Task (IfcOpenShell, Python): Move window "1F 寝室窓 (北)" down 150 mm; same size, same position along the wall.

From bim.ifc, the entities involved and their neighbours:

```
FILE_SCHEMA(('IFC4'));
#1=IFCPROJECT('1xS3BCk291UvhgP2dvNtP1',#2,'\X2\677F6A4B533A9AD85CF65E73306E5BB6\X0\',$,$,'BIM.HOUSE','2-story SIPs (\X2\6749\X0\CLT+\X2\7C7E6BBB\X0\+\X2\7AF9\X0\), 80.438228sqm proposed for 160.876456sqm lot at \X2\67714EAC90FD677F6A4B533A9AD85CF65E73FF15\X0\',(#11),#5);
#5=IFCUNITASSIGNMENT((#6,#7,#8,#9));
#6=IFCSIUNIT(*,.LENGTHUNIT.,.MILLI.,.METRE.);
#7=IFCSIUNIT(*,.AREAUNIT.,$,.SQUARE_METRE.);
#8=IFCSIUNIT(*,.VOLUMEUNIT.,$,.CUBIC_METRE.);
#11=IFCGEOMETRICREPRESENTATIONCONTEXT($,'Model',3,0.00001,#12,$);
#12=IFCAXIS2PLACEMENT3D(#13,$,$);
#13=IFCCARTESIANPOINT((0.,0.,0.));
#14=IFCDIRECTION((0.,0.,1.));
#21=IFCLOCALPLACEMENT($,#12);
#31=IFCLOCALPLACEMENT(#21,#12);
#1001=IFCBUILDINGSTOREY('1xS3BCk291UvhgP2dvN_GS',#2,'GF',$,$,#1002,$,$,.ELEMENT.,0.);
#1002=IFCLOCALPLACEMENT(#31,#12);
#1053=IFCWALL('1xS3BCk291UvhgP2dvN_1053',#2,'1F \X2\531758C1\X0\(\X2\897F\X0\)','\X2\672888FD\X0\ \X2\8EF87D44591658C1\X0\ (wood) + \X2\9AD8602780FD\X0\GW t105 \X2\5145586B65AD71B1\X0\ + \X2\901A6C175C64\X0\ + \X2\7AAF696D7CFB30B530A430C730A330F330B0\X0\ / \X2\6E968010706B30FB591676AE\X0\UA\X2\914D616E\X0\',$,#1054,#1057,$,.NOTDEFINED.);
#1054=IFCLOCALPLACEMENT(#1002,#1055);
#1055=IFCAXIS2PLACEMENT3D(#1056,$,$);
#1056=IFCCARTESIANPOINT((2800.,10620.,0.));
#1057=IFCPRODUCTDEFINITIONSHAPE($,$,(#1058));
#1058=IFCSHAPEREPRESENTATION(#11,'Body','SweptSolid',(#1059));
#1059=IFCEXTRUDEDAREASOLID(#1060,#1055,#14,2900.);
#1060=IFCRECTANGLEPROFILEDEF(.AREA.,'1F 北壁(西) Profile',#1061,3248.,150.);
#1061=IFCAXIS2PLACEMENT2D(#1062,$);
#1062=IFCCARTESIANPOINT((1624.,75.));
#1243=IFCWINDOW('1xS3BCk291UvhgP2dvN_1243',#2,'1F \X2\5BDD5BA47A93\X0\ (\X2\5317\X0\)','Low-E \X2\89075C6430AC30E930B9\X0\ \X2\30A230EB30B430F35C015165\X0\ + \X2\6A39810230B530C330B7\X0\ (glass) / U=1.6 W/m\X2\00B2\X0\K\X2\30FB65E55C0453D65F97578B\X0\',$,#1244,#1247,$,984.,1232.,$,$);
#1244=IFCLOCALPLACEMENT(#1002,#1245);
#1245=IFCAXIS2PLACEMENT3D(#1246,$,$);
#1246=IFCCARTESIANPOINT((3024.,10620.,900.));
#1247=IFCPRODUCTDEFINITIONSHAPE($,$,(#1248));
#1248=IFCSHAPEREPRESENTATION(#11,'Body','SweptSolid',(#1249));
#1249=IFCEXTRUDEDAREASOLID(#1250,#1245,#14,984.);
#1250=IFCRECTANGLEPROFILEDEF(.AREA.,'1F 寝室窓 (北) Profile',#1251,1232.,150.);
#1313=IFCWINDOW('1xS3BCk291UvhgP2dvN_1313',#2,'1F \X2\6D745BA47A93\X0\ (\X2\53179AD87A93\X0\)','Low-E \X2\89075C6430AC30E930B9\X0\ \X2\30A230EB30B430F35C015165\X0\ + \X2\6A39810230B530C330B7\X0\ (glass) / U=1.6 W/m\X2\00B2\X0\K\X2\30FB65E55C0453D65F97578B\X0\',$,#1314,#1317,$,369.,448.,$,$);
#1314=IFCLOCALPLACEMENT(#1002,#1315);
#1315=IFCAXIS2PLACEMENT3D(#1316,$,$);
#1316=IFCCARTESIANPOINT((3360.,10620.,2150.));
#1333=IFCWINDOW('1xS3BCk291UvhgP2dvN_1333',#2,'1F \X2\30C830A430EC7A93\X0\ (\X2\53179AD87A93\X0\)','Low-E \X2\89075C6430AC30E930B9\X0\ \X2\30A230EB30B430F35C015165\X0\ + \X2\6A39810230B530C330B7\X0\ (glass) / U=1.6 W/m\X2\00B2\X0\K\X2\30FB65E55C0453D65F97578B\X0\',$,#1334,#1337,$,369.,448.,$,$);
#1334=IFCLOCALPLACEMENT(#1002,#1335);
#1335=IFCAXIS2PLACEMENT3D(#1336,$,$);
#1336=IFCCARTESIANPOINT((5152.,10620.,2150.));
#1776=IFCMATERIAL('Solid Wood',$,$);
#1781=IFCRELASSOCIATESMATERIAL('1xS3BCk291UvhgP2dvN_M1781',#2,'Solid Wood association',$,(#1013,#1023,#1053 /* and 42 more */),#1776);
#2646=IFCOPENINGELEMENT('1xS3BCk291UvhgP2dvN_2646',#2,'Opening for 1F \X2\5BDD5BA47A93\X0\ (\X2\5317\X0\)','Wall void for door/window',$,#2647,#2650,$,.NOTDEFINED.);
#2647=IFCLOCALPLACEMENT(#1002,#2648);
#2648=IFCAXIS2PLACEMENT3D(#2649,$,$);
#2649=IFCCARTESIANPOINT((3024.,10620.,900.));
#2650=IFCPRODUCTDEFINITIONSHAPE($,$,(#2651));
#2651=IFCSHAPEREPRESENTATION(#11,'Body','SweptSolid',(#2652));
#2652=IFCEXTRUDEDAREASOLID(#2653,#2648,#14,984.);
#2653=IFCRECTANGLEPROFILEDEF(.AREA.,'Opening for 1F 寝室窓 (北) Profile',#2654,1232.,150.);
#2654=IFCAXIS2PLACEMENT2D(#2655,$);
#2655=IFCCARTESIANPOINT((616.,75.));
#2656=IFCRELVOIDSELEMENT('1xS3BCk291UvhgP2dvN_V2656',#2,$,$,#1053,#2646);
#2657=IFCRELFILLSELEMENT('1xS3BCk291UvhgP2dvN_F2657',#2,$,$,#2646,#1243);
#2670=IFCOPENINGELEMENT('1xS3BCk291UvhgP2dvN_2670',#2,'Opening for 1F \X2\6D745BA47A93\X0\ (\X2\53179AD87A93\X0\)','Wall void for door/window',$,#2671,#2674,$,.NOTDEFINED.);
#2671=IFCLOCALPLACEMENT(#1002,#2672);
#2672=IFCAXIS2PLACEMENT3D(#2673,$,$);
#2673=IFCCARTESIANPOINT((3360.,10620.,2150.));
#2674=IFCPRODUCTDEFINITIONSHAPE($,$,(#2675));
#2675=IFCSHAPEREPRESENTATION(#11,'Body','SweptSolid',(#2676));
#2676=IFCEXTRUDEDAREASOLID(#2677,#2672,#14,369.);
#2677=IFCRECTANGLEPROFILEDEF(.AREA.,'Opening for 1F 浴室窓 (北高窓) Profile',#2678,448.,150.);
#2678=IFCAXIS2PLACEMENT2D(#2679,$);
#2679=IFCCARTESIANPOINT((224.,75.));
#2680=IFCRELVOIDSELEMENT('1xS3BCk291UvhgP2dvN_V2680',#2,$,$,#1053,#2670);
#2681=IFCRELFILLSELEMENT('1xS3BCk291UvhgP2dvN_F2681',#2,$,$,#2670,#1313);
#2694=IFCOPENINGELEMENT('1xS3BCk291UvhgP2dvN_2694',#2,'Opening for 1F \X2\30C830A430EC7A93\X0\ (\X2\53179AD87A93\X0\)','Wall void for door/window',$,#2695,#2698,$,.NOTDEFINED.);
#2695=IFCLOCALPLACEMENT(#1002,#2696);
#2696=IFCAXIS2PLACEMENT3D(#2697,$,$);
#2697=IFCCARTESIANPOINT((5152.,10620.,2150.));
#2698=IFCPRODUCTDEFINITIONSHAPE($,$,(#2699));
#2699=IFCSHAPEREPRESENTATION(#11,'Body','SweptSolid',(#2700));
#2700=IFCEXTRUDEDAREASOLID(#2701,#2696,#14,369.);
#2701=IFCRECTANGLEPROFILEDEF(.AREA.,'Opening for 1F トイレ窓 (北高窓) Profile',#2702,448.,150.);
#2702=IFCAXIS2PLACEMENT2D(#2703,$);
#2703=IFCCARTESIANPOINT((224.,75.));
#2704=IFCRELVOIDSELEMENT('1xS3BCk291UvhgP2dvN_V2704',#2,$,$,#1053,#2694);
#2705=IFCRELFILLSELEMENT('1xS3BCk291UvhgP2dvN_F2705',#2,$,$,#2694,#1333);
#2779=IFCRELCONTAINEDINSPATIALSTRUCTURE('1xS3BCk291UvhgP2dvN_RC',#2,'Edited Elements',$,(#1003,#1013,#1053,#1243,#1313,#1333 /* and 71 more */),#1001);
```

```python
import numpy as np
import ifcopenshell
import ifcopenshell.api.geometry
import ifcopenshell.util.placement
import ifcopenshell.util.unit

model = ifcopenshell.open("bim.ifc")
unit_scale = ifcopenshell.util.unit.calculate_unit_scale(model)

window = model.by_guid("1xS3BCk291UvhgP2dvN_1243")
opening = window.FillsVoids[0].RelatingOpeningElement
dz = -0.15 / unit_scale

shift = np.array([0.0, 0.0, dz])
# The window is not placed relative to its opening, so move both.
for product in (opening, window):
    matrix = ifcopenshell.util.placement.get_local_placement(product.ObjectPlacement)
    matrix[:3, 3] += shift
    ifcopenshell.api.geometry.edit_object_placement(model, product=product, matrix=matrix, is_si=False)

print(f"moved by {dz * unit_scale:+.3f} m")

model.write("bim-out.ifc")
```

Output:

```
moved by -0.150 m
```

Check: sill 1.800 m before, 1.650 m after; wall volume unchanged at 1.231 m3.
